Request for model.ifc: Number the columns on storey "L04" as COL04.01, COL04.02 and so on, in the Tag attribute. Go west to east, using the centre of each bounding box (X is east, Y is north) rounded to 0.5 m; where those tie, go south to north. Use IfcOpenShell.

First a look at what the model holds.

```python
import ifcopenshell
import ifcopenshell.util.element
import ifcopenshell.util.placement

model = ifcopenshell.open("model.ifc")
print(model.schema)
storey = next(s for s in model.by_type("IfcBuildingStorey") if s.Name == "L04")
columns = [e for e in ifcopenshell.util.element.get_decomposition(storey) if e.is_a("IfcColumn")]
for e in sorted(columns, key=lambda e: e.id()):
    origin = ifcopenshell.util.placement.get_local_placement(e.ObjectPlacement)[:3, 3]
    print(e.id(), e.Tag, e.Name, origin.round(2) + 0.0, sep=" | ")
```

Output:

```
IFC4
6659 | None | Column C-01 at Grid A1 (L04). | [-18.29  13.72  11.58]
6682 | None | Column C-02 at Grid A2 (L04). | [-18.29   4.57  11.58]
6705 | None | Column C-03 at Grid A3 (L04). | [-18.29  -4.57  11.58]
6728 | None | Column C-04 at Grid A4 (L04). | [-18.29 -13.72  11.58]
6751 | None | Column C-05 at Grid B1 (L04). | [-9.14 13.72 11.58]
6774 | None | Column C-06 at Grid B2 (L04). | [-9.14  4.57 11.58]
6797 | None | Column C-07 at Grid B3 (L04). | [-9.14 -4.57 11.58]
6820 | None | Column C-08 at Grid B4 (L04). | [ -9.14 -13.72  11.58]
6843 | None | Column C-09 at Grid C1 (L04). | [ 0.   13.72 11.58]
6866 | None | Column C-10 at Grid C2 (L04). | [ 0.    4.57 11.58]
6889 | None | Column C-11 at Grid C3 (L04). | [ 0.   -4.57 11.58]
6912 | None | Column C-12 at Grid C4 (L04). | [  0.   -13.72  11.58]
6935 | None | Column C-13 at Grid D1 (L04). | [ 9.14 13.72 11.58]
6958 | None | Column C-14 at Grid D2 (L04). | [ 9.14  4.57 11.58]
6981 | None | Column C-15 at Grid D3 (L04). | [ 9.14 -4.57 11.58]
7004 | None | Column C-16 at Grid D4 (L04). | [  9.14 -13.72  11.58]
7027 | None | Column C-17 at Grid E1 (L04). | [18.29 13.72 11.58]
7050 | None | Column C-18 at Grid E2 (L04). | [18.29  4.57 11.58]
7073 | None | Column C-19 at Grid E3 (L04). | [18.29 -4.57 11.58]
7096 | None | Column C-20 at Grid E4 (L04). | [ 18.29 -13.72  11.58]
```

```python
import ifcopenshell
import ifcopenshell.geom
import ifcopenshell.util.element
import ifcopenshell.util.shape

model = ifcopenshell.open("model.ifc")
settings = ifcopenshell.geom.settings()
settings.set("use-world-coords", True)


def centre(element):
    shape = ifcopenshell.geom.create_shape(settings, element)
    return ifcopenshell.util.shape.get_bbox_centroid(shape.geometry)


storey = next(s for s in model.by_type("IfcBuildingStorey") if s.Name == "L04")
columns = [e for e in ifcopenshell.util.element.get_decomposition(storey) if e.is_a("IfcColumn")]

# Insertion points can sit at a corner or the storey origin, so sort by the geometry (in metres).
centres = {e: centre(e) for e in columns}
columns.sort(key=lambda e: (round(centres[e][0] / 0.5), centres[e][1]))

for i, e in enumerate(columns, start=1):
    number = f"COL04.{i:02d}"
    e.Tag = number
    print(e.id(), number)

model.write("model_rev.ifc")
```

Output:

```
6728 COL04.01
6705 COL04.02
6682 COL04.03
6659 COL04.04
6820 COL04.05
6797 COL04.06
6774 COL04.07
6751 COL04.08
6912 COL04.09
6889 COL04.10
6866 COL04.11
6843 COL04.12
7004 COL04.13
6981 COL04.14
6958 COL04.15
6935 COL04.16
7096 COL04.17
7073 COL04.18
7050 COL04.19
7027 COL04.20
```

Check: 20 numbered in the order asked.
